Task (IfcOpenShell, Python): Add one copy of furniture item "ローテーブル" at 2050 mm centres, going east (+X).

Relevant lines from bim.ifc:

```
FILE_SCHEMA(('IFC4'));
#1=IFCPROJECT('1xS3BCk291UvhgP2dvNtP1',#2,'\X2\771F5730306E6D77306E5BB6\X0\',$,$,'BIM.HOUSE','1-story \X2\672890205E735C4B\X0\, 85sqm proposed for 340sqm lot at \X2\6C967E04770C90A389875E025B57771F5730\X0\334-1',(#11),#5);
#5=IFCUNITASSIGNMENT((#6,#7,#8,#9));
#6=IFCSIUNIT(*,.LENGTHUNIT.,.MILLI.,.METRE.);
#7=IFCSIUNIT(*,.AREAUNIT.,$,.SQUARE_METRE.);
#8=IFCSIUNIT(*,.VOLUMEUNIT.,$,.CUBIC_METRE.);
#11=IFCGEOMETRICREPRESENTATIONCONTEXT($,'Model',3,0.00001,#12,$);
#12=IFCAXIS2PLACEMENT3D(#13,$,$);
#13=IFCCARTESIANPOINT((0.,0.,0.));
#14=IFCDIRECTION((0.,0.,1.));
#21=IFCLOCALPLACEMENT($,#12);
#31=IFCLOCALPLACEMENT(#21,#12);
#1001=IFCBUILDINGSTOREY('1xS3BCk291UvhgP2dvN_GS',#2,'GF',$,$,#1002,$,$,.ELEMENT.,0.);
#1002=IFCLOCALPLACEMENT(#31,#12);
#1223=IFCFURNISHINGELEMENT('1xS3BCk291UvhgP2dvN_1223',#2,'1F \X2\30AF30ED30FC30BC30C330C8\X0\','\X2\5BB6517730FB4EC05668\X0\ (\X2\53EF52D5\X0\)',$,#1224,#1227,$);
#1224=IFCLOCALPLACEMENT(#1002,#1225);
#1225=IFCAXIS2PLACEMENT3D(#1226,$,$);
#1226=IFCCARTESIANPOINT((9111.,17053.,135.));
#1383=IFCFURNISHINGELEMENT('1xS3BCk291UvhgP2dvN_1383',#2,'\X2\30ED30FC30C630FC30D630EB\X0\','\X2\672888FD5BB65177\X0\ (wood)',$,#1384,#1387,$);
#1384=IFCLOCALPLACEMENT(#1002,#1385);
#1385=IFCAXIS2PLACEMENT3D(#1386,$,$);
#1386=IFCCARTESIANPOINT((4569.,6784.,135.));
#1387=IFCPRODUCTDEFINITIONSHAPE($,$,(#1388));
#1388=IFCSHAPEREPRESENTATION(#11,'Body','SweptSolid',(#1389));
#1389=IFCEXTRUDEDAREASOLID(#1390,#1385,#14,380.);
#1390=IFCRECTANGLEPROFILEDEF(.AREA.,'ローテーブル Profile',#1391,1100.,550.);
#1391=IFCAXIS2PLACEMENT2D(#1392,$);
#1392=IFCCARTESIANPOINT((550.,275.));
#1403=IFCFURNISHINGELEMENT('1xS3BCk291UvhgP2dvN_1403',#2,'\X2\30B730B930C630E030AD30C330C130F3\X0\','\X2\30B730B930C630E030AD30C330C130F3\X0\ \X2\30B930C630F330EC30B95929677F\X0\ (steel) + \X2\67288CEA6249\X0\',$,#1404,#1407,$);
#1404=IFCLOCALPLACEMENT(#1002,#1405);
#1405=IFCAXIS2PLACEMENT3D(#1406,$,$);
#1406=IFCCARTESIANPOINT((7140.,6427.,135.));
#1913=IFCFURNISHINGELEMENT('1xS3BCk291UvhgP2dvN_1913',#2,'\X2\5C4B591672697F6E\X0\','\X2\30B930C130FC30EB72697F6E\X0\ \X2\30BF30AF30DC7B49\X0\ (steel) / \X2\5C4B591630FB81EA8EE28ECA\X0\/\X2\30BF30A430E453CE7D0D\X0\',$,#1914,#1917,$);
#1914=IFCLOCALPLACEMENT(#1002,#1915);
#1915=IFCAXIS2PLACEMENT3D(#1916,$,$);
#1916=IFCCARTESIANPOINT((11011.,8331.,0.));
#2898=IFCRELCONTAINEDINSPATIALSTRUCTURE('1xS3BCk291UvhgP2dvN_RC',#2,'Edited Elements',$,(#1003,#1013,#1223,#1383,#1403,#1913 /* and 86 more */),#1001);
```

```python
import numpy as np
import ifcopenshell
import ifcopenshell.api.geometry
import ifcopenshell.api.root
import ifcopenshell.util.element
import ifcopenshell.util.placement
import ifcopenshell.util.unit

model = ifcopenshell.open("bim.ifc")
unit_scale = ifcopenshell.util.unit.calculate_unit_scale(model)


def reuse_history(source, copy):
    """copy_class also copies each property set's owner history, people and application; keep the originals."""
    for rel in copy.IsDefinedBy:
        if rel.is_a("IfcRelDefinesByProperties") and (history := rel.RelatingPropertyDefinition.OwnerHistory):
            rel.RelatingPropertyDefinition.OwnerHistory = source.OwnerHistory
            ifcopenshell.util.element.remove_deep2(model, history)


source = model.by_id(1383)
base = ifcopenshell.util.placement.get_local_placement(source.ObjectPlacement)
step = np.array([1.0, 0.0, 0.0]) * 2.05 / unit_scale

for i in range(1, 2):
    copy = ifcopenshell.api.root.copy_class(model, product=source)
    copy.Representation = ifcopenshell.util.element.copy_deep(
        model, source.Representation, exclude=["IfcGeometricRepresentationContext", "IfcRepresentationMap"]
    )
    reuse_history(source, copy)
    matrix = base.copy()
    matrix[:3, 3] += i * step
    print("added at", matrix[:3, 3].round(3) + 0.0)
    ifcopenshell.api.geometry.edit_object_placement(model, product=copy, matrix=matrix, is_si=False)

model.write("bim-out.ifc")
```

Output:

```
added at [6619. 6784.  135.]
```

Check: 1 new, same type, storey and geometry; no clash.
